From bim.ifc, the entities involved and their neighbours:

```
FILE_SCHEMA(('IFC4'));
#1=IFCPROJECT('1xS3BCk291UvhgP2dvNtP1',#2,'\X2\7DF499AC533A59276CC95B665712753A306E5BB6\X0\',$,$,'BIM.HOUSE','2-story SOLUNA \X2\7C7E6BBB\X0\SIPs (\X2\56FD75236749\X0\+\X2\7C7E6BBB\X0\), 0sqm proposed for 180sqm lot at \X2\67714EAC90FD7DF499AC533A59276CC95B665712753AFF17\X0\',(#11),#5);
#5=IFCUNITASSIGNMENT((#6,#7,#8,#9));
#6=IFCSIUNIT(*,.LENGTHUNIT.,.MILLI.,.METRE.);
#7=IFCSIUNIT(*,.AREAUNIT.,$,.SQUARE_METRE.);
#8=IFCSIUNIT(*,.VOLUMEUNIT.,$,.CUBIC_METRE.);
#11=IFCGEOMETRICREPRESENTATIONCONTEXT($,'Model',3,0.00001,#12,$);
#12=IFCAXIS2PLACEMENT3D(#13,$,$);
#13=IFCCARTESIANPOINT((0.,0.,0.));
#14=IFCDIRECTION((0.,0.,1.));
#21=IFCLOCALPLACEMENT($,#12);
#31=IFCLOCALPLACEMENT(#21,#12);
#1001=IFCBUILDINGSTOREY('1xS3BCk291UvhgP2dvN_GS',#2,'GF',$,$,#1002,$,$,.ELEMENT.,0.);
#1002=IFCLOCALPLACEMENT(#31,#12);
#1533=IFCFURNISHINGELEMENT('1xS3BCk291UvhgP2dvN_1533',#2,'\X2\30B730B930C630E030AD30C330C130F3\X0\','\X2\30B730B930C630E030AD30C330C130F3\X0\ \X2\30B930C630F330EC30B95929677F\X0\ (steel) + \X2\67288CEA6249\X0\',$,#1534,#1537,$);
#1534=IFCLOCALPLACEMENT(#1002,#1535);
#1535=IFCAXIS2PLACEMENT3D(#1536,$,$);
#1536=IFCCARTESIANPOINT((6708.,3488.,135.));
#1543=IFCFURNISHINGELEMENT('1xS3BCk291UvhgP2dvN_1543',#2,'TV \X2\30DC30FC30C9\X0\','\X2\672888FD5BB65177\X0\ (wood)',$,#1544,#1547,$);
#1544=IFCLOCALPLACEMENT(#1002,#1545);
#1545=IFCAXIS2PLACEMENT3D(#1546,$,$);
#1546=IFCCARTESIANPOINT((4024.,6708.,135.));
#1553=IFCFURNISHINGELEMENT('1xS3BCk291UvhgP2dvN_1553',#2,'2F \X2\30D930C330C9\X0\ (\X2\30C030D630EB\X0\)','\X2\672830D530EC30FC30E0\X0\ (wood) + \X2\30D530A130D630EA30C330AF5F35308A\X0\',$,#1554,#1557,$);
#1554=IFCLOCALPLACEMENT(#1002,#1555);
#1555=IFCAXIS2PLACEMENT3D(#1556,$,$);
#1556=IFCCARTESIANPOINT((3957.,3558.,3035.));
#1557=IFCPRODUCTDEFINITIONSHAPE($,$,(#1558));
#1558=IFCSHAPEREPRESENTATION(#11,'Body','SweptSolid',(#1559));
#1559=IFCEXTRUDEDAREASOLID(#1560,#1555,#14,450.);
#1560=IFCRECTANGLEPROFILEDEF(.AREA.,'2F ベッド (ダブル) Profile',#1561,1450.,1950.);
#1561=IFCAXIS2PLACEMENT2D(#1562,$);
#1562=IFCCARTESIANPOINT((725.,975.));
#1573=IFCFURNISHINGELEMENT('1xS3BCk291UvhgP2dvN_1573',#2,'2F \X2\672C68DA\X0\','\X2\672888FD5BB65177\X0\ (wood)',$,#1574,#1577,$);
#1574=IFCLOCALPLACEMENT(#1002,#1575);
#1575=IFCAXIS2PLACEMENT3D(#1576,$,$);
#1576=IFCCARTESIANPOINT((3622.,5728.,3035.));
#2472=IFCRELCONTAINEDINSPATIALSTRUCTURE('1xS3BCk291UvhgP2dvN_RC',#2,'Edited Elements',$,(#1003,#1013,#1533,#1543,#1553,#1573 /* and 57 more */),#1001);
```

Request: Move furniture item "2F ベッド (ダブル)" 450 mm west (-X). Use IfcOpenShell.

```python
import ifcopenshell
import ifcopenshell.api.geometry
import ifcopenshell.util.placement
import ifcopenshell.util.unit

model = ifcopenshell.open("bim.ifc")
unit_scale = ifcopenshell.util.unit.calculate_unit_scale(model)

item = model.by_guid("1xS3BCk291UvhgP2dvN_1553")
matrix = ifcopenshell.util.placement.get_local_placement(item.ObjectPlacement)
matrix[0, 3] -= 0.45 / unit_scale
ifcopenshell.api.geometry.edit_object_placement(model, product=item, matrix=matrix, is_si=False)

print(ifcopenshell.util.placement.get_local_placement(item.ObjectPlacement).round(3) + 0.0)

model.write("bim_rev.ifc")
```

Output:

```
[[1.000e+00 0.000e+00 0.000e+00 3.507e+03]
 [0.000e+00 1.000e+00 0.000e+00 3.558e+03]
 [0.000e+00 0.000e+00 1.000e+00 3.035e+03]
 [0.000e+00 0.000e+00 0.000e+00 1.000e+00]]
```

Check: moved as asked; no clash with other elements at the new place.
